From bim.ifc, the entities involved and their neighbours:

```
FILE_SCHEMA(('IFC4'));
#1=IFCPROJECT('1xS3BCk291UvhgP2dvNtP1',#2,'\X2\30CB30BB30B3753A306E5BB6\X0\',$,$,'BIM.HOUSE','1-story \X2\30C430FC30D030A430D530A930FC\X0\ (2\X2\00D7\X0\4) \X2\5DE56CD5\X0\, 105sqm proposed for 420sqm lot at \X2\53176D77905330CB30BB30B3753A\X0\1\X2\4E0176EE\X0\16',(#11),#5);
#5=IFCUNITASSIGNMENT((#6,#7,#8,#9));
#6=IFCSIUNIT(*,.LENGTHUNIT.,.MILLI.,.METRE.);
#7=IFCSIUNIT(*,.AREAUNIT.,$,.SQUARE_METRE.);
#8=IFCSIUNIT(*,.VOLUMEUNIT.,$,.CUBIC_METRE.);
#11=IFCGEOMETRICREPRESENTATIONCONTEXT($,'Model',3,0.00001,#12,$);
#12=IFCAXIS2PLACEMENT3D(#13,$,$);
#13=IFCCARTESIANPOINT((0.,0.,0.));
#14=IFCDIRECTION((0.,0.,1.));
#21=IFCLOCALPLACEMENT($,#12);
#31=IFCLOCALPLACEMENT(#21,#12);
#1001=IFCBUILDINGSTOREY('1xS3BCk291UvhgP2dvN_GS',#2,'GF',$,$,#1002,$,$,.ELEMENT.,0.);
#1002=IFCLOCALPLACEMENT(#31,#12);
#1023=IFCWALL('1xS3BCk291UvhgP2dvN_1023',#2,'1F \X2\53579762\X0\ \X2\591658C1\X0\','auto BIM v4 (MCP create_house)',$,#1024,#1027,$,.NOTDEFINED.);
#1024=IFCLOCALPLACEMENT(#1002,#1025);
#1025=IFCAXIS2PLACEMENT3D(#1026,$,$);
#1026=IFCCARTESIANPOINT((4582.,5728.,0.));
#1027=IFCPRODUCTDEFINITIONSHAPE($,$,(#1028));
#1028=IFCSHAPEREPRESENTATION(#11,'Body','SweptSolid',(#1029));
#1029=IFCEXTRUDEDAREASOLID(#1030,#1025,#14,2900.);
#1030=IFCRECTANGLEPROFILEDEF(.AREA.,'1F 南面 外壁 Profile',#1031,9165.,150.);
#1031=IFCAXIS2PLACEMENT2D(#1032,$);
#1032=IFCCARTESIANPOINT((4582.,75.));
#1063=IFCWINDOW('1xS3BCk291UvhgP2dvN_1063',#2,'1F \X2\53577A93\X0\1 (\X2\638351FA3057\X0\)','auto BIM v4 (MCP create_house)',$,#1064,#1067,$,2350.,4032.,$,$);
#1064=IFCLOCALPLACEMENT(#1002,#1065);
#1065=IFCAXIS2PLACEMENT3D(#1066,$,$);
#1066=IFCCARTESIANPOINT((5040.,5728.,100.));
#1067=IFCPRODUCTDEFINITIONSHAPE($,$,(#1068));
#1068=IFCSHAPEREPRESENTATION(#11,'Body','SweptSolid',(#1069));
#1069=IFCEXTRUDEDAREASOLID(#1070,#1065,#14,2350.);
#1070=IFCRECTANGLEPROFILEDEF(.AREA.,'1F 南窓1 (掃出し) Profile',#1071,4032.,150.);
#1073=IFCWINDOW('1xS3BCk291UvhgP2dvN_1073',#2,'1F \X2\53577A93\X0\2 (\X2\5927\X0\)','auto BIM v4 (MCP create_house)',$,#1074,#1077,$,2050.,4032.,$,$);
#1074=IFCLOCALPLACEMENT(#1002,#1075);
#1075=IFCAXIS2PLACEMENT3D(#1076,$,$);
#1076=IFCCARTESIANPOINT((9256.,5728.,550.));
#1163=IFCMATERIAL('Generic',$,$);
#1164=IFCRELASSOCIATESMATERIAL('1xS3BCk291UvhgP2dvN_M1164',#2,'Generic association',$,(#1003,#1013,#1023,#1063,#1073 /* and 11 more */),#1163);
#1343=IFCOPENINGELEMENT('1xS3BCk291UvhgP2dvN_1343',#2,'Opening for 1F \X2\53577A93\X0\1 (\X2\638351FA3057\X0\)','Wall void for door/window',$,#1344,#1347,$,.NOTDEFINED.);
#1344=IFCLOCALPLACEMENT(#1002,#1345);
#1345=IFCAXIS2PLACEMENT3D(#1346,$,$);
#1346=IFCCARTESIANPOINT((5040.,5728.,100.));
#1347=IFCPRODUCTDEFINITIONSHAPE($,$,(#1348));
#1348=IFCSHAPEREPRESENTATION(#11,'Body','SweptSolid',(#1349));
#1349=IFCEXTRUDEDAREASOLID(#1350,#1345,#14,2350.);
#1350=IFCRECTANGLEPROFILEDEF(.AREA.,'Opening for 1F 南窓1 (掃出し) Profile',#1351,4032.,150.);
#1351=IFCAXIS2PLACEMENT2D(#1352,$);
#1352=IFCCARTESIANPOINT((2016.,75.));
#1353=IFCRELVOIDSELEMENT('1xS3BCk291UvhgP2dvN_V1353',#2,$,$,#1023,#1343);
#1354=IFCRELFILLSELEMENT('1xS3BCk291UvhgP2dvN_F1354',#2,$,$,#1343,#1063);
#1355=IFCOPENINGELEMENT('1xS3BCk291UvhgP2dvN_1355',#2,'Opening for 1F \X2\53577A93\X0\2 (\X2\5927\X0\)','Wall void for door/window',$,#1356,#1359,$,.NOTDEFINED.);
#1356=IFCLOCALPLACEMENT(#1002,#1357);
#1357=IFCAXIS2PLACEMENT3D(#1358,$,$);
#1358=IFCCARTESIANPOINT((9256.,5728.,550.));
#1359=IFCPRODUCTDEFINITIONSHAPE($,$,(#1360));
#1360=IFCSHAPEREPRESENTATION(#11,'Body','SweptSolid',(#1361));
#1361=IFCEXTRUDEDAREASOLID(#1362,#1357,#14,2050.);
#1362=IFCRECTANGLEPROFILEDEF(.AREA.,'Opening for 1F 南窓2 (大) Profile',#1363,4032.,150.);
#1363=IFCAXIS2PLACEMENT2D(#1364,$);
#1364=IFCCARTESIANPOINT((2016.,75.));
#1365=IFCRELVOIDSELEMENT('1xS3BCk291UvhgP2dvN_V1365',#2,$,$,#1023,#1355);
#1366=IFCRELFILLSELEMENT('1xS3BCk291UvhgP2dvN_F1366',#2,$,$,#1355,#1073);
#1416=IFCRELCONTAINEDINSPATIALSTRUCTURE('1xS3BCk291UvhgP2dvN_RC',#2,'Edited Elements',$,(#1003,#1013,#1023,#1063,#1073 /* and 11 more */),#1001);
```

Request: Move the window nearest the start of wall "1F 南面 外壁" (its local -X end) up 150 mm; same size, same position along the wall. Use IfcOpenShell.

```python
import numpy as np
import ifcopenshell
import ifcopenshell.api.geometry
import ifcopenshell.util.placement
import ifcopenshell.util.unit

model = ifcopenshell.open("bim.ifc")
unit_scale = ifcopenshell.util.unit.calculate_unit_scale(model)

window = model.by_guid("1xS3BCk291UvhgP2dvN_1063")
opening = window.FillsVoids[0].RelatingOpeningElement
dz = 150.0

shift = np.array([0.0, 0.0, dz])
# The window is not placed relative to its opening, so move both.
for product in (opening, window):
    matrix = ifcopenshell.util.placement.get_local_placement(product.ObjectPlacement)
    matrix[:3, 3] += shift
    ifcopenshell.api.geometry.edit_object_placement(model, product=product, matrix=matrix, is_si=False)

print(f"moved by {dz * unit_scale:+.3f} m")

model.write("bim_updated.ifc")
```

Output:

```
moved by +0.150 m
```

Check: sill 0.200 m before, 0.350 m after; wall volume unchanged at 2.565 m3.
